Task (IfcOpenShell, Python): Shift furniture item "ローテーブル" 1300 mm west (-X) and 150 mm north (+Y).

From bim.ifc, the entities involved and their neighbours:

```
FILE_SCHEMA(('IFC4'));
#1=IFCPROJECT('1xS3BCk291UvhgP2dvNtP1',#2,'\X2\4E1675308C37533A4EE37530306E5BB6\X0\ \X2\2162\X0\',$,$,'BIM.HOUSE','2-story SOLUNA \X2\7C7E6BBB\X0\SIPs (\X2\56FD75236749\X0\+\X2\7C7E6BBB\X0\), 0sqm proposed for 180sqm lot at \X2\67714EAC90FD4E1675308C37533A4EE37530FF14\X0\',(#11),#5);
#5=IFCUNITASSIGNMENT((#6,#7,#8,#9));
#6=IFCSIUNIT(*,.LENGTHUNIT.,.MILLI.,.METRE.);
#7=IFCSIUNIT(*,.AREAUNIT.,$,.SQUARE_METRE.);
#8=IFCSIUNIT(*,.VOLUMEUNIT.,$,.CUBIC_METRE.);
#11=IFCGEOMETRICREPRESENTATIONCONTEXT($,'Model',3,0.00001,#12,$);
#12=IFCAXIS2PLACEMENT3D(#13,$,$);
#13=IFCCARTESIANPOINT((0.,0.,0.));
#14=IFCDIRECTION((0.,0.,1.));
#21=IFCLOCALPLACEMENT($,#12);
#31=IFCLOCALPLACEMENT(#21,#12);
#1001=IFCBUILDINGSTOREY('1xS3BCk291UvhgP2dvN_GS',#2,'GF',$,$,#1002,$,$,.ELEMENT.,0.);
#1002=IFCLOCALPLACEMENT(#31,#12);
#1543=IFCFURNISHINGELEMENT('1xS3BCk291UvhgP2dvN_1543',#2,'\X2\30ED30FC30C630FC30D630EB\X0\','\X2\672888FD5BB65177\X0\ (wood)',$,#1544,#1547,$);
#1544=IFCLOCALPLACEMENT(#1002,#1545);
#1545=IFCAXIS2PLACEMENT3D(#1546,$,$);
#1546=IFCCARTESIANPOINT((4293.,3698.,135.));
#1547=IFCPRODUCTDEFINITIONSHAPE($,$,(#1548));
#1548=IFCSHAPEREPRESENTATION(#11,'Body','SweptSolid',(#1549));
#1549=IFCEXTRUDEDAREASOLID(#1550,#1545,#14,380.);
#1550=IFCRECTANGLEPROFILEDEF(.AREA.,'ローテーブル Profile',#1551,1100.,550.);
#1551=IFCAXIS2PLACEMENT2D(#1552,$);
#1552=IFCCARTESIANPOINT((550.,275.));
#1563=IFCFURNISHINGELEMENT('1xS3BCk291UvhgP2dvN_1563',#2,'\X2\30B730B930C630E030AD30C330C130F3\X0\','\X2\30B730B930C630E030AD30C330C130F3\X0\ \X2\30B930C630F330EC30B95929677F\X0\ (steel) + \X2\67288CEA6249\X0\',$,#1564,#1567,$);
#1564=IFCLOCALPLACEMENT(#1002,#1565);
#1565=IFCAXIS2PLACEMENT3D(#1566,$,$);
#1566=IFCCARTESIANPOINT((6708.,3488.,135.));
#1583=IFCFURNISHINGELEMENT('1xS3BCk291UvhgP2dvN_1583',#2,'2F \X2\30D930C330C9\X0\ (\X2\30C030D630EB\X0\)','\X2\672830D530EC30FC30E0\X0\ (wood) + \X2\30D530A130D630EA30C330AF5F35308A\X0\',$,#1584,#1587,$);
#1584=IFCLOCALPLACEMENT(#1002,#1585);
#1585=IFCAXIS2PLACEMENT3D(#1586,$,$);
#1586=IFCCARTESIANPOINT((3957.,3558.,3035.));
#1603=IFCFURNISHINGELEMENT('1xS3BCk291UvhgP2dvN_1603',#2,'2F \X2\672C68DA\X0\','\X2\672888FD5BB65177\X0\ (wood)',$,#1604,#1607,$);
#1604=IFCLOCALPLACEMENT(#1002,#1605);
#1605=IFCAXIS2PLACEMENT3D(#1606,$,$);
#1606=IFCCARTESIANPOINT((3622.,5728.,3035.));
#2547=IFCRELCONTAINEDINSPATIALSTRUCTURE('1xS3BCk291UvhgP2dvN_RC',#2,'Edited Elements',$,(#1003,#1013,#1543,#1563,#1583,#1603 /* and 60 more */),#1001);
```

```python
import ifcopenshell
import ifcopenshell.api.geometry
import ifcopenshell.util.placement
import ifcopenshell.util.unit

model = ifcopenshell.open("bim.ifc")
unit_scale = ifcopenshell.util.unit.calculate_unit_scale(model)

item = model.by_guid("1xS3BCk291UvhgP2dvN_1543")
matrix = ifcopenshell.util.placement.get_local_placement(item.ObjectPlacement)
matrix[0, 3] -= 1.3 / unit_scale
matrix[1, 3] += 0.15 / unit_scale
ifcopenshell.api.geometry.edit_object_placement(model, product=item, matrix=matrix, is_si=False)

print(ifcopenshell.util.placement.get_local_placement(item.ObjectPlacement).round(3) + 0.0)

model.write("bim_v2.ifc")
```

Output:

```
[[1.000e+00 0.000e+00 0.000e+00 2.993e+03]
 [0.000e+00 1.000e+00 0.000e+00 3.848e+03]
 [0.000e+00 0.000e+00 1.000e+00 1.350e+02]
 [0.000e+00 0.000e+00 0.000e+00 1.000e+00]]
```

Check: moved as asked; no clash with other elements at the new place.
